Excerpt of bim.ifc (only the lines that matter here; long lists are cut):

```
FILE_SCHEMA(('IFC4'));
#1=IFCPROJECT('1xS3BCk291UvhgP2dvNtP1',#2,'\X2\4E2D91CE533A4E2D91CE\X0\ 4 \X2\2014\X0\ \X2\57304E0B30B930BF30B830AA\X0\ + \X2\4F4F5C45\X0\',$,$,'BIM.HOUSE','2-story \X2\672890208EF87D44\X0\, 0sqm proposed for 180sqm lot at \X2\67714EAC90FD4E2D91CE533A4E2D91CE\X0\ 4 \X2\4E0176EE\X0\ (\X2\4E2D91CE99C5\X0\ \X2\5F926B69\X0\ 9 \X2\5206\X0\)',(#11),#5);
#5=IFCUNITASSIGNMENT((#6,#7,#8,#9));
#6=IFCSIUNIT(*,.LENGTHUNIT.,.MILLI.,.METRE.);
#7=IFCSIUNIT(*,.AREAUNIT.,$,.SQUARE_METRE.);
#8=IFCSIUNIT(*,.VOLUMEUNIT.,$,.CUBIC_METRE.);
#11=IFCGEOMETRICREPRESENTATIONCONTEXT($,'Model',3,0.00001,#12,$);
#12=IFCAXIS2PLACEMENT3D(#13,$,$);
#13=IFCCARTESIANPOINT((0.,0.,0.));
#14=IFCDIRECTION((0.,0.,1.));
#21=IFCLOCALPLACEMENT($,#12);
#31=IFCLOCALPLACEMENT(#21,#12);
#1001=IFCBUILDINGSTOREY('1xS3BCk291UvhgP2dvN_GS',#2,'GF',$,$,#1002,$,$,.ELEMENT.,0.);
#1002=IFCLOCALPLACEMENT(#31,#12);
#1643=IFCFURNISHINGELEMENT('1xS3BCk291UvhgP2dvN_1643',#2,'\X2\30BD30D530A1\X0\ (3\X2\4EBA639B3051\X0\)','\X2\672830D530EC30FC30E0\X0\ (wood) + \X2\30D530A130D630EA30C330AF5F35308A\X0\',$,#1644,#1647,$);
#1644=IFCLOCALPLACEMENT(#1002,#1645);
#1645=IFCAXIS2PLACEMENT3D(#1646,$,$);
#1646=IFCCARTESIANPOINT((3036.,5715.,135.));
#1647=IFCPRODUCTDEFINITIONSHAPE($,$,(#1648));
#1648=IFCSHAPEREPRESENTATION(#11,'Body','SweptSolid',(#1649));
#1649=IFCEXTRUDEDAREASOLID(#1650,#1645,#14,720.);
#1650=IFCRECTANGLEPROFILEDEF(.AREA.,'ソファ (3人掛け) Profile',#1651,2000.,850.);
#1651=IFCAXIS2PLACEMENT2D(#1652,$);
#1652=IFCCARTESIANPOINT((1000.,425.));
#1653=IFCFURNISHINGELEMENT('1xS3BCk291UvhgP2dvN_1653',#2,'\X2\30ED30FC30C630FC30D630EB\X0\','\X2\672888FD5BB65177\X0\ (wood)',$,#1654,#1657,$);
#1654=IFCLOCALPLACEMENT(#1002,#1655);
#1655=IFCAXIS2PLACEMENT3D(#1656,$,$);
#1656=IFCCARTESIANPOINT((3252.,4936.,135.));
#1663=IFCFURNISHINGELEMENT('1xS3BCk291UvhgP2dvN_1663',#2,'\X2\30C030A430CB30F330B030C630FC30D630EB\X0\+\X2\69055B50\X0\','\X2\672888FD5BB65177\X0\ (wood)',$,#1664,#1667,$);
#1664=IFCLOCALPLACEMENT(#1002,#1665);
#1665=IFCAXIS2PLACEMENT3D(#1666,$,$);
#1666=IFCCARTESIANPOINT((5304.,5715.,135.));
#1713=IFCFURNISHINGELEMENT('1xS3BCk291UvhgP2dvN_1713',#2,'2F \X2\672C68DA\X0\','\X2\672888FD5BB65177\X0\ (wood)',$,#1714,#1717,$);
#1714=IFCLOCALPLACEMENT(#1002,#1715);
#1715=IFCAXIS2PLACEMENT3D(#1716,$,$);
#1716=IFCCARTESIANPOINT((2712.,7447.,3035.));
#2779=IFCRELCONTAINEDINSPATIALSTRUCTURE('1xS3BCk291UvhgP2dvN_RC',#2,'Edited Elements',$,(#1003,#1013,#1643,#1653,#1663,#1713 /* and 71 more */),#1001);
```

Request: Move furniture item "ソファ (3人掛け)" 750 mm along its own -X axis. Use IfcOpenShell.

```python
import ifcopenshell
import ifcopenshell.api.geometry
import ifcopenshell.util.placement

model = ifcopenshell.open("bim.ifc")

item = model.by_guid("1xS3BCk291UvhgP2dvN_1643")
matrix = ifcopenshell.util.placement.get_local_placement(item.ObjectPlacement)
matrix[:3, 3] -= matrix[:3, 0] * 750.0
ifcopenshell.api.geometry.edit_object_placement(model, product=item, matrix=matrix, is_si=False)

print(ifcopenshell.util.placement.get_local_placement(item.ObjectPlacement).round(3) + 0.0)

model.write("bim_v2.ifc")
```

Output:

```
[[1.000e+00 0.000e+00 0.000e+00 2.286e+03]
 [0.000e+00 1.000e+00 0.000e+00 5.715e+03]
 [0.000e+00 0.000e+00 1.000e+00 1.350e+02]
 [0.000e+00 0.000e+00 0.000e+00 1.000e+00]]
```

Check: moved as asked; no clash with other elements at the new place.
